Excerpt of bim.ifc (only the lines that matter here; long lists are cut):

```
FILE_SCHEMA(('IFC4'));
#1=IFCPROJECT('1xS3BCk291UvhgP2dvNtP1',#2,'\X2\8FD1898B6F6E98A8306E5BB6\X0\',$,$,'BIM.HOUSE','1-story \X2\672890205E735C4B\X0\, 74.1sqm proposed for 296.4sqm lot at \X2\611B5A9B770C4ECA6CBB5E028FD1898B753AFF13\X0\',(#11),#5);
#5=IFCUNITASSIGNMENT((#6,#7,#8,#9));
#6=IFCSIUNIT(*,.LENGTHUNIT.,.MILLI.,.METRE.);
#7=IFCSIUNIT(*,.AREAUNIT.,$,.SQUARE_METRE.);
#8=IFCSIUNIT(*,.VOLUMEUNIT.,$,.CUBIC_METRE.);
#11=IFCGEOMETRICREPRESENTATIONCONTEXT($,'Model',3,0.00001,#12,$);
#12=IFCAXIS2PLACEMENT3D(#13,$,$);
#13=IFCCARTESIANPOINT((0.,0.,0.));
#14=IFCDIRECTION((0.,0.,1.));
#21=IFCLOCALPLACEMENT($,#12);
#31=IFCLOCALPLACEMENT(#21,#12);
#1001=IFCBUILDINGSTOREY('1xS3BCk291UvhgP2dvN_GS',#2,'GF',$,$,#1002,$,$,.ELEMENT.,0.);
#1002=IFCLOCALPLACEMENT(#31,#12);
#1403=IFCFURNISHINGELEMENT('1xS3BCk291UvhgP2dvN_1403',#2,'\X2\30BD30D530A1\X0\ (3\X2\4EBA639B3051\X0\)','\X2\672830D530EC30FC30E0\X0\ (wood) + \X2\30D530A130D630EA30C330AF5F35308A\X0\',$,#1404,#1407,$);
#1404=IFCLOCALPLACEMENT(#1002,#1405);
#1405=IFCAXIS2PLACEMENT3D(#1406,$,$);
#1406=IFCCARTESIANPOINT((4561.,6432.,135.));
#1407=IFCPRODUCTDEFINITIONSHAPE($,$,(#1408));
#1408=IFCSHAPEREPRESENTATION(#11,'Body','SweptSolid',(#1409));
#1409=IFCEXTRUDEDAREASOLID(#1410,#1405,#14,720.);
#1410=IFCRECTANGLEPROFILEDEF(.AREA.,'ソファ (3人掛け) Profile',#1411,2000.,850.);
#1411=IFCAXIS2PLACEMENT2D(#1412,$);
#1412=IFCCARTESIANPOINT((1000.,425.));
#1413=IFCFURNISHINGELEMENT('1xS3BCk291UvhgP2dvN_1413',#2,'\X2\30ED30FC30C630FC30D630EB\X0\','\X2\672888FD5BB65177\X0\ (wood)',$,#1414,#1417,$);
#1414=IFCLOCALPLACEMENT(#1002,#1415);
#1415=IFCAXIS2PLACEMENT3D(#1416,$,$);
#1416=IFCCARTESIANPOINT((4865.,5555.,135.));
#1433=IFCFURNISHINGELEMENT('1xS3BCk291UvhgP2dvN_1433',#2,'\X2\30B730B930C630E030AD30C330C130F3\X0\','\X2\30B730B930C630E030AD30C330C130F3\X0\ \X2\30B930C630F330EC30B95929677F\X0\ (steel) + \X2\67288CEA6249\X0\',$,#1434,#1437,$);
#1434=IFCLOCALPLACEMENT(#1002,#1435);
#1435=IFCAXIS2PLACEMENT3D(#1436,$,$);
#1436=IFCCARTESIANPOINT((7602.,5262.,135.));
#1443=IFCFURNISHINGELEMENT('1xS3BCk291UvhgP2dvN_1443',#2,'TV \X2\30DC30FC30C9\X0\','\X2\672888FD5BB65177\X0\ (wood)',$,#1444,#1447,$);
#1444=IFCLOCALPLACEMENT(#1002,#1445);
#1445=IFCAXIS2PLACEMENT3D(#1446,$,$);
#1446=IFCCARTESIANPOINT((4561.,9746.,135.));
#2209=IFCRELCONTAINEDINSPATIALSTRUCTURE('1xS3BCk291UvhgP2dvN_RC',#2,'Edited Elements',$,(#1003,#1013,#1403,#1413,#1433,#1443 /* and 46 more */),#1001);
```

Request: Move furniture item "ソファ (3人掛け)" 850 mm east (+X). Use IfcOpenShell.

```python
import ifcopenshell
import ifcopenshell.api.geometry
import ifcopenshell.util.placement

model = ifcopenshell.open("bim.ifc")

item = model.by_guid("1xS3BCk291UvhgP2dvN_1403")
matrix = ifcopenshell.util.placement.get_local_placement(item.ObjectPlacement)
matrix[0, 3] += 850.0
ifcopenshell.api.geometry.edit_object_placement(model, product=item, matrix=matrix, is_si=False)

print(ifcopenshell.util.placement.get_local_placement(item.ObjectPlacement).round(3) + 0.0)

model.write("bim_edited.ifc")
```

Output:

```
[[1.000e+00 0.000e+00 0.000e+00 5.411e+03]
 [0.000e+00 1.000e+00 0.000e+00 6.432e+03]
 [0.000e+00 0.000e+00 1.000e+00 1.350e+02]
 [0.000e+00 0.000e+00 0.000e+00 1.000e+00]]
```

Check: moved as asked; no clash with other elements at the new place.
